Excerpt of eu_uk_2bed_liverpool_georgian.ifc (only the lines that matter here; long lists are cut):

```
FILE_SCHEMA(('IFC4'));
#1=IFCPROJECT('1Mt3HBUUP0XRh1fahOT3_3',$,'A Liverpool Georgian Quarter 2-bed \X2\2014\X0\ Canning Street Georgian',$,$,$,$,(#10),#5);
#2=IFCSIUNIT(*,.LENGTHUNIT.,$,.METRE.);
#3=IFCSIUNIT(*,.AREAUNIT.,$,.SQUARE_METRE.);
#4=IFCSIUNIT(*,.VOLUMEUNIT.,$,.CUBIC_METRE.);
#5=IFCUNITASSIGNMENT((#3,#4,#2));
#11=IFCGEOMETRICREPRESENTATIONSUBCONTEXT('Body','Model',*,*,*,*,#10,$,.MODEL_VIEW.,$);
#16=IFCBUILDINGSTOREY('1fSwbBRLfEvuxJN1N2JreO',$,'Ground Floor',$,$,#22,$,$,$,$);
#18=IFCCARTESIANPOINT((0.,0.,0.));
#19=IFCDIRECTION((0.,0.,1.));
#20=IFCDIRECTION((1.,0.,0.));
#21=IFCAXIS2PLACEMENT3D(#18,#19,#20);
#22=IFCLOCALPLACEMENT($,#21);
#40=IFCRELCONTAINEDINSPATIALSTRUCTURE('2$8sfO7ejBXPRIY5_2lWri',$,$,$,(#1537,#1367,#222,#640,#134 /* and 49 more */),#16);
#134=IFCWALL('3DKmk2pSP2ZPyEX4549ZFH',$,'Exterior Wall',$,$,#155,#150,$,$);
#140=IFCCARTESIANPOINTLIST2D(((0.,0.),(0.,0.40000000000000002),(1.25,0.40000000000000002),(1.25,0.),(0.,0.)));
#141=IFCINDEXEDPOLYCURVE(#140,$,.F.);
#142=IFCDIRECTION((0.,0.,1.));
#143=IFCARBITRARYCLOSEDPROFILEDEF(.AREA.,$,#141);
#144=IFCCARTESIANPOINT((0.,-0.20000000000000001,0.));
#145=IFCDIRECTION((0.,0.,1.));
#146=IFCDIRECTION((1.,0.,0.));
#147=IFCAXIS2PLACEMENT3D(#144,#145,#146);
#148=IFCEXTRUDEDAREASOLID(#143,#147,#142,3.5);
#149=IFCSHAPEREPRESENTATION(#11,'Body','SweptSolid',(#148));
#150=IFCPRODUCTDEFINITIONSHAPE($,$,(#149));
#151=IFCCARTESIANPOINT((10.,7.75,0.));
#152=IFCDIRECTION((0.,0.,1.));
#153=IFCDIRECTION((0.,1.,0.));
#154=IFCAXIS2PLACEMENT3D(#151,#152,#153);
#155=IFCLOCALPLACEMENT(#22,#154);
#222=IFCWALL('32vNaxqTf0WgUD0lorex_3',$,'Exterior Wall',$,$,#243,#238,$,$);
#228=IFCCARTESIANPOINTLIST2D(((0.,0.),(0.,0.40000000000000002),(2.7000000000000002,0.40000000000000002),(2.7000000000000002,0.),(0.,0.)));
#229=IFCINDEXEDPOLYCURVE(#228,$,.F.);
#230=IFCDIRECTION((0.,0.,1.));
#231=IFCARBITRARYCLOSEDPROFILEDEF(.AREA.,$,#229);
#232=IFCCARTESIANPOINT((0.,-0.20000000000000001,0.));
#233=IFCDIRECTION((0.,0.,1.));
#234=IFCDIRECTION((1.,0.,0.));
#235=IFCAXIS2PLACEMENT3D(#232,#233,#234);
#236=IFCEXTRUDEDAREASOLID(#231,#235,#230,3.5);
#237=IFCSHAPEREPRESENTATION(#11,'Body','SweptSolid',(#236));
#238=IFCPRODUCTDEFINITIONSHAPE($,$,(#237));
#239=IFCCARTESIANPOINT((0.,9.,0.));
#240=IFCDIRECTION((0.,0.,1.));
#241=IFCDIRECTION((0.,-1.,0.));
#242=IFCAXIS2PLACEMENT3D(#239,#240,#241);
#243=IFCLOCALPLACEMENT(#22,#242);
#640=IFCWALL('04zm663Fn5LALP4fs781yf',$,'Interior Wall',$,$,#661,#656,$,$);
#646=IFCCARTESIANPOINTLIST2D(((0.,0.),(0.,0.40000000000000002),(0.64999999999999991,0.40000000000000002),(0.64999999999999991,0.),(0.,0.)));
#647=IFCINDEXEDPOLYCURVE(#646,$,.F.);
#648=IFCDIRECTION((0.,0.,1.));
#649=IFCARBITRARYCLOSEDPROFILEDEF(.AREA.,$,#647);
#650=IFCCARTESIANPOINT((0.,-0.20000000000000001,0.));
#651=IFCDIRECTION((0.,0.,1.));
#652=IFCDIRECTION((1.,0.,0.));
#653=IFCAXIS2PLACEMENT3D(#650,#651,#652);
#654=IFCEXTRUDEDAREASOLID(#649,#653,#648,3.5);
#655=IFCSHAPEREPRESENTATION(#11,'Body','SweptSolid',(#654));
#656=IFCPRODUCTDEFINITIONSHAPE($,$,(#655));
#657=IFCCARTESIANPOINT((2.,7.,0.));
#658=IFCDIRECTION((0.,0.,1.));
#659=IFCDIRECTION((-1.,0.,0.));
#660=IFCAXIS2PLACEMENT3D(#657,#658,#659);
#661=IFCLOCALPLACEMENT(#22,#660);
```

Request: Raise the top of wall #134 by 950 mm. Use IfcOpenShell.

```python
import ifcopenshell
import ifcopenshell.geom
import ifcopenshell.util.representation
import ifcopenshell.util.shape
import ifcopenshell.util.unit

model = ifcopenshell.open("eu_uk_2bed_liverpool_georgian.ifc")
unit_scale = ifcopenshell.util.unit.calculate_unit_scale(model)
settings = ifcopenshell.geom.settings()


def volume(element):
    """Net volume in cubic metres, openings subtracted."""
    shape = ifcopenshell.geom.create_shape(settings, element)
    return ifcopenshell.util.shape.get_volume(shape.geometry)


wall = model.by_guid("3DKmk2pSP2ZPyEX4549ZFH")
before = volume(wall)

body = ifcopenshell.util.representation.get_representation(wall, "Model", "Body")
solid = body.Items[0]
old_height = solid.Depth
solid.Depth += 0.95 / unit_scale
after = volume(wall)

print(f"height {old_height:g} -> {solid.Depth:g}, volume {before:.3f} -> {after:.3f} m3")

model.write("eu_uk_2bed_liverpool_georgian_updated.ifc")
```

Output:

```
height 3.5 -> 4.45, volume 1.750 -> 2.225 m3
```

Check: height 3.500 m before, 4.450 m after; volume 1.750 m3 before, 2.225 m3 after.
